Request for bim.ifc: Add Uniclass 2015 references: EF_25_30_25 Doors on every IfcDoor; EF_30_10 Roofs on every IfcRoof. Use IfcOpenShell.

First a look at what the model holds.

```python
import ifcopenshell

model = ifcopenshell.open("bim.ifc")
print(model.schema)
print("classifications:", [c.Name for c in model.by_type("IfcClassification")])
for ifc_class in ("IfcDoor", "IfcRoof", "IfcStair", "IfcWall", "IfcWindow"):
    print(ifc_class, len(model.by_type(ifc_class)))
```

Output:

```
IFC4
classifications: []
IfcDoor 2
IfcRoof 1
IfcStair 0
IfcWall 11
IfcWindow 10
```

```python
import ifcopenshell
import ifcopenshell.api.classification

model = ifcopenshell.open("bim.ifc")

system = ifcopenshell.api.classification.add_classification(model, classification="Uniclass 2015")

codes = {
    "IfcDoor": ("EF_25_30_25", "Doors"),
    "IfcRoof": ("EF_30_10", "Roofs"),
}
for ifc_class, (code, name) in codes.items():
    products = model.by_type(ifc_class)
    ifcopenshell.api.classification.add_reference(
        model, products=products, classification=system, identification=code, name=name
    )
    print(code, len(products))

model.write("bim_v2.ifc")
```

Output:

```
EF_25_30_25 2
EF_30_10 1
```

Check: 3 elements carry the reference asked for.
